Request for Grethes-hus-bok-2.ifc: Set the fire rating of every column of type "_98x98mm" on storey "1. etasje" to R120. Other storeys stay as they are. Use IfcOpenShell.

First a look at what the model holds.

```python
import ifcopenshell
import ifcopenshell.util.element

model = ifcopenshell.open("Grethes-hus-bok-2.ifc")
print(model.schema)
storey = next(s for s in model.by_type("IfcBuildingStorey") if s.Name == "1. etasje")
columns = [e for e in ifcopenshell.util.element.get_decomposition(storey) if e.is_a("IfcColumn")]
seen = {}
for e in columns:
    element_type = ifcopenshell.util.element.get_type(e)
    key = (element_type.Name if element_type != e and element_type else None, ifcopenshell.util.element.get_pset(e, "Pset_ColumnCommon", "FireRating"))
    seen[key] = seen.get(key, 0) + 1
for (name, value), count in sorted(seen.items(), key=str):
    print(count, "x", name, "|", value)
```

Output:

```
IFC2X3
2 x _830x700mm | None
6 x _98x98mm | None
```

```python
import ifcopenshell
import ifcopenshell.api.pset
import ifcopenshell.util.element

model = ifcopenshell.open("Grethes-hus-bok-2.ifc")

storey = next(s for s in model.by_type("IfcBuildingStorey") if s.Name == "1. etasje")
columns = [e for e in ifcopenshell.util.element.get_decomposition(storey) if e.is_a("IfcColumn")]

count = 0
for e in columns:
    element_type = ifcopenshell.util.element.get_type(e)
    if element_type in (None, e) or element_type.Name != "_98x98mm":
        continue
    # add_pset returns the element's existing set when there is one.
    pset = ifcopenshell.api.pset.add_pset(model, product=e, name="Pset_ColumnCommon")
    ifcopenshell.api.pset.edit_pset(model, pset=pset, properties={"FireRating": "R120"})
    count += 1

print(count, "columns updated")

model.write("Grethes-hus-bok-2_updated.ifc")
```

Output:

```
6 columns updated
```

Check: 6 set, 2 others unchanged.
